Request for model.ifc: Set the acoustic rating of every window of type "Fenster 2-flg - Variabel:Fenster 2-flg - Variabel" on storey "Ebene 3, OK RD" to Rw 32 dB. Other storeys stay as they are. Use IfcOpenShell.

First a look at what the model holds.

```python
import ifcopenshell
import ifcopenshell.util.element

model = ifcopenshell.open("model.ifc")
print(model.schema)
storey = next(s for s in model.by_type("IfcBuildingStorey") if s.Name == "Ebene 3, OK RD")
windows = [e for e in ifcopenshell.util.element.get_decomposition(storey) if e.is_a("IfcWindow")]
seen = {}
for e in windows:
    element_type = ifcopenshell.util.element.get_type(e)
    key = (element_type.Name if element_type != e and element_type else None, ifcopenshell.util.element.get_pset(e, "Pset_WindowCommon", "AcousticRating"))
    seen[key] = seen.get(key, 0) + 1
for (name, value), count in sorted(seen.items(), key=str):
    print(count, "x", name, "|", value)
```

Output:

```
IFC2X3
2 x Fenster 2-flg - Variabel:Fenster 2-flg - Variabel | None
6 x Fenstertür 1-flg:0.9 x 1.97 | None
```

```python
import ifcopenshell
import ifcopenshell.api.pset
import ifcopenshell.util.element

model = ifcopenshell.open("model.ifc")

storey = next(s for s in model.by_type("IfcBuildingStorey") if s.Name == "Ebene 3, OK RD")
windows = [e for e in ifcopenshell.util.element.get_decomposition(storey) if e.is_a("IfcWindow")]

count = 0
for e in windows:
    element_type = ifcopenshell.util.element.get_type(e)
    if element_type in (None, e) or element_type.Name != "Fenster 2-flg - Variabel:Fenster 2-flg - Variabel":
        continue
    # add_pset returns the element's existing set when there is one.
    pset = ifcopenshell.api.pset.add_pset(model, product=e, name="Pset_WindowCommon")
    ifcopenshell.api.pset.edit_pset(model, pset=pset, properties={"AcousticRating": "Rw 32 dB"})
    count += 1

print(count, "windows updated")

model.write("model_updated.ifc")
```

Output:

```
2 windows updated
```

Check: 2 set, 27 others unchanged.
